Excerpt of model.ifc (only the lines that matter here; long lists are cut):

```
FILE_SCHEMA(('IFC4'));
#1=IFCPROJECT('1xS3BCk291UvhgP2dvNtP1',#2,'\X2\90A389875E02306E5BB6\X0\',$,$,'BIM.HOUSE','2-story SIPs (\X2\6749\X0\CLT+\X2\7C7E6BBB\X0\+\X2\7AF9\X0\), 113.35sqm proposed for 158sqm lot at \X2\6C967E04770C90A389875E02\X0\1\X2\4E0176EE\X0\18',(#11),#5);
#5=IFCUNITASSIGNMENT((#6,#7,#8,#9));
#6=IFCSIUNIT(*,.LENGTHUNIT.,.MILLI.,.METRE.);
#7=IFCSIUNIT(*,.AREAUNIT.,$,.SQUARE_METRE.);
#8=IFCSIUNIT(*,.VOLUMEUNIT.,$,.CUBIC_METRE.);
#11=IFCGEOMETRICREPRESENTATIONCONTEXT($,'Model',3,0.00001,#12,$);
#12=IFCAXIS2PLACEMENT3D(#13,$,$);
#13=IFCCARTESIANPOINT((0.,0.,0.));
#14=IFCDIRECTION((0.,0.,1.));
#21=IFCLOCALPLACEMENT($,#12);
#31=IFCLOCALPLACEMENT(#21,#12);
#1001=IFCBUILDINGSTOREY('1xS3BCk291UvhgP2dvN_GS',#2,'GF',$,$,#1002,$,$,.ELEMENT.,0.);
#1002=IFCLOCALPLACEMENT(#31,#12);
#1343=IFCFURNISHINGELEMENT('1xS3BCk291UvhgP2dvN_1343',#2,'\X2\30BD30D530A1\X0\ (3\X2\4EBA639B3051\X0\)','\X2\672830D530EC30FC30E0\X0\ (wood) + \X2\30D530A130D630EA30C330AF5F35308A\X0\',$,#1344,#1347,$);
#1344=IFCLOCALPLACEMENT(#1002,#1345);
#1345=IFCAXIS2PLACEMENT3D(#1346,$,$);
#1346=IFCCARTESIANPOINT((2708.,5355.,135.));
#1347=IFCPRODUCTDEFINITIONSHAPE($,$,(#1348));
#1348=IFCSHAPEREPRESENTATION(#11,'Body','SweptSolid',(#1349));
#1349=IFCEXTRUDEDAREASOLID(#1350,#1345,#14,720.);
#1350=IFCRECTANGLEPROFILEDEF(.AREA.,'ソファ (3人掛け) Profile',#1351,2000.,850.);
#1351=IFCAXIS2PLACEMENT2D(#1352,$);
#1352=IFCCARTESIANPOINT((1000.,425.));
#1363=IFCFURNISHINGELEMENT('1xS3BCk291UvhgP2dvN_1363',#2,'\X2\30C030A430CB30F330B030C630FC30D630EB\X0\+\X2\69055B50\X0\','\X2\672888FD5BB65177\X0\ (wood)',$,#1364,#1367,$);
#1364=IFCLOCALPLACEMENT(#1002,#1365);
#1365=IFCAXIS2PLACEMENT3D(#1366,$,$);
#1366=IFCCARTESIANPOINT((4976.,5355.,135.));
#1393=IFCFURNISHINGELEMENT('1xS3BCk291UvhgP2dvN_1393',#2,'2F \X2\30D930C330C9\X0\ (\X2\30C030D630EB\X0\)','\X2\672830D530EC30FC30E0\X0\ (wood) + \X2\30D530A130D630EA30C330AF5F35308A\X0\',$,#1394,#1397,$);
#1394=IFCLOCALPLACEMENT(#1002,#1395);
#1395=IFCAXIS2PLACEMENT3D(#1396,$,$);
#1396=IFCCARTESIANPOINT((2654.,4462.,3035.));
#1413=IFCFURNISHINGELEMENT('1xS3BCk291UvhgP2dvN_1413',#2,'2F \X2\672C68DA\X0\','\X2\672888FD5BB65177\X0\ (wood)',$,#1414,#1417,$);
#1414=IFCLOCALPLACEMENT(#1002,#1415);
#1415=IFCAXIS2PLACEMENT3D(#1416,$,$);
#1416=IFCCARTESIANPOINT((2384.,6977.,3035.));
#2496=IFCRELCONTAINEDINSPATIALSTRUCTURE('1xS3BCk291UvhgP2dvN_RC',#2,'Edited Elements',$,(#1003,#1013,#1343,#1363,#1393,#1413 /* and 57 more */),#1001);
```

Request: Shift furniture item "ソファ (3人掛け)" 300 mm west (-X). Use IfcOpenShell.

```python
import ifcopenshell
import ifcopenshell.api.geometry
import ifcopenshell.util.placement
import ifcopenshell.util.unit

model = ifcopenshell.open("model.ifc")
unit_scale = ifcopenshell.util.unit.calculate_unit_scale(model)

item = model.by_guid("1xS3BCk291UvhgP2dvN_1343")
matrix = ifcopenshell.util.placement.get_local_placement(item.ObjectPlacement)
matrix[0, 3] -= 0.3 / unit_scale
ifcopenshell.api.geometry.edit_object_placement(model, product=item, matrix=matrix, is_si=False)

print(ifcopenshell.util.placement.get_local_placement(item.ObjectPlacement).round(3) + 0.0)

model.write("model_updated.ifc")
```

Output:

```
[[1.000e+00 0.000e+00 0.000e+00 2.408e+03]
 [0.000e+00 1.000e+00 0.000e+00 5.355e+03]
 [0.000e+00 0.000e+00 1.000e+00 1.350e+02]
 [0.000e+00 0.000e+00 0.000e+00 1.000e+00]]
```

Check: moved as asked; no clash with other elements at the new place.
